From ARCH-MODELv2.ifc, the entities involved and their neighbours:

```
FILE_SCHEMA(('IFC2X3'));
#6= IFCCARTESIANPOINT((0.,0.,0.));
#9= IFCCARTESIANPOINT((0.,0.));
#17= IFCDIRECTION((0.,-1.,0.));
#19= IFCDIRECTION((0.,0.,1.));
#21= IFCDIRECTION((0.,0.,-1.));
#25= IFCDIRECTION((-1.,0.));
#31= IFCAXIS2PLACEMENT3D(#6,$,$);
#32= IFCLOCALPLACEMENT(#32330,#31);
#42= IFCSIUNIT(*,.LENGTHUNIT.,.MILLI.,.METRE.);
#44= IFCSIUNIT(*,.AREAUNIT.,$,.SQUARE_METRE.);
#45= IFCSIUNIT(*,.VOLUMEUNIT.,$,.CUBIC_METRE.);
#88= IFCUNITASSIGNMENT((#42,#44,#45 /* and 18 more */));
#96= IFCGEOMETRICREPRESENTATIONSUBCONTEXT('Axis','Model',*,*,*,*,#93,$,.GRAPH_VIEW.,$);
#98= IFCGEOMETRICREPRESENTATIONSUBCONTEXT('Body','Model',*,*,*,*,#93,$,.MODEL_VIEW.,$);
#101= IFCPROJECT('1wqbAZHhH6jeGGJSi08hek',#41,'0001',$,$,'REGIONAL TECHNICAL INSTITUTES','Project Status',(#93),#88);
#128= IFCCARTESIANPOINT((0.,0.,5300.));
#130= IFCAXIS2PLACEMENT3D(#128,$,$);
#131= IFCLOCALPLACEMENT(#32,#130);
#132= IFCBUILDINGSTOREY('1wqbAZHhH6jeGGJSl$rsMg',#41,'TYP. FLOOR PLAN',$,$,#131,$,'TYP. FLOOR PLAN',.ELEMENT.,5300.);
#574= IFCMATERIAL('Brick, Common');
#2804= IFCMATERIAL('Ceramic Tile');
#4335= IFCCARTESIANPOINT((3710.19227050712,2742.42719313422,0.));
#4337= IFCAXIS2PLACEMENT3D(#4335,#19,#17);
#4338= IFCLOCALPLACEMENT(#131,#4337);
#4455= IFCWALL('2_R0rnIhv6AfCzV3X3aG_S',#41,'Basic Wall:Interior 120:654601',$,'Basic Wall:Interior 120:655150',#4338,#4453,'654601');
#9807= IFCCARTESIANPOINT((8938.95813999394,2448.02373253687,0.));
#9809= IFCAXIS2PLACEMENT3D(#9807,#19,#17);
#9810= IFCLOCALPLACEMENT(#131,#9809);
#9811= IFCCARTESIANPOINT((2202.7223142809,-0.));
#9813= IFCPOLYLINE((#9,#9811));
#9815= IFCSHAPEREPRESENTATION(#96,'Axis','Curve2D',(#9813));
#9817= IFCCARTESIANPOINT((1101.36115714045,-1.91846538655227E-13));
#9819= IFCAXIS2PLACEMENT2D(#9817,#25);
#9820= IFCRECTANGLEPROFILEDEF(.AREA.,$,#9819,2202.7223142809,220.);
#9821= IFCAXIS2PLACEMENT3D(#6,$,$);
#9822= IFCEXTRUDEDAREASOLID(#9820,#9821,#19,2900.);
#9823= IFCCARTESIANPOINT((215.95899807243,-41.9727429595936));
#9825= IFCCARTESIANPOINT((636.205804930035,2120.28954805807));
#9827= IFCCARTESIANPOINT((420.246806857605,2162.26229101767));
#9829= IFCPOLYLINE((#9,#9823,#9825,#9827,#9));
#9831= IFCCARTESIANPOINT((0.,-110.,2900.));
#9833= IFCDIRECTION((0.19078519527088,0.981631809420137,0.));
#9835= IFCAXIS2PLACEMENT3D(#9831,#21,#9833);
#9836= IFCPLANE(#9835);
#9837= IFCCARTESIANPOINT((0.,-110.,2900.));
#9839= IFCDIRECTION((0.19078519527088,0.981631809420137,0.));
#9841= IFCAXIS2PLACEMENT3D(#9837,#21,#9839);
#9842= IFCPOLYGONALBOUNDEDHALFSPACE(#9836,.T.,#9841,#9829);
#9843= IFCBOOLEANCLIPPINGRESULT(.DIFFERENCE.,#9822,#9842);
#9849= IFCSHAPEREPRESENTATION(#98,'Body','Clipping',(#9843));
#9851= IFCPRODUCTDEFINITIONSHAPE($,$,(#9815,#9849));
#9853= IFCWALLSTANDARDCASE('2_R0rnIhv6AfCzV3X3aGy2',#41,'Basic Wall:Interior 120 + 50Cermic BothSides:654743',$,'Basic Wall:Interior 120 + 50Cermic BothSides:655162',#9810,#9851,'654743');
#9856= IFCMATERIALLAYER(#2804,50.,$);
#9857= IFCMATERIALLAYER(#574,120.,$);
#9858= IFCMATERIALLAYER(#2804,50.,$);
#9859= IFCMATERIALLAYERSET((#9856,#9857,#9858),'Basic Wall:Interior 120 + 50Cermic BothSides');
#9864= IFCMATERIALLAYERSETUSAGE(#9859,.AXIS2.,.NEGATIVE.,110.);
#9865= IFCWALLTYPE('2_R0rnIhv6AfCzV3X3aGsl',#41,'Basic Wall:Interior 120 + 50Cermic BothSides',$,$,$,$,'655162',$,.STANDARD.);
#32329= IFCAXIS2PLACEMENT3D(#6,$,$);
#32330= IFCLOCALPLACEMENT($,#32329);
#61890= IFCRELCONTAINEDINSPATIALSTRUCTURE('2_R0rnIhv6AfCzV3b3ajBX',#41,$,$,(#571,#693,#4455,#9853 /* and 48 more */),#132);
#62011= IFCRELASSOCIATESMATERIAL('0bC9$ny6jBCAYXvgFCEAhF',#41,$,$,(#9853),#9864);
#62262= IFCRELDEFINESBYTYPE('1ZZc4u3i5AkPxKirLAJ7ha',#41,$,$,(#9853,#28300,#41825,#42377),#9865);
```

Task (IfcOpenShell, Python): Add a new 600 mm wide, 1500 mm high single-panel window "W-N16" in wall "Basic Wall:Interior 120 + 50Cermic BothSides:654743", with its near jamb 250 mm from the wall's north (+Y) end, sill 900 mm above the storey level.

```python
import numpy as np
import ifcopenshell
import ifcopenshell.api.feature
import ifcopenshell.api.geometry
import ifcopenshell.api.root
import ifcopenshell.api.spatial
import ifcopenshell.api.type
import ifcopenshell.geom
import ifcopenshell.util.element
import ifcopenshell.util.placement
import ifcopenshell.util.representation
import ifcopenshell.util.shape
import ifcopenshell.util.unit

model = ifcopenshell.open("ARCH-MODELv2.ifc")
unit_scale = ifcopenshell.util.unit.calculate_unit_scale(model)
settings = ifcopenshell.geom.settings()


def volume(element):
    """Net volume in cubic metres, openings subtracted."""
    shape = ifcopenshell.geom.create_shape(settings, element)
    return ifcopenshell.util.shape.get_volume(shape.geometry)


wall = model.by_guid("2_R0rnIhv6AfCzV3X3aGy2")
storey = ifcopenshell.util.element.get_container(wall, ifc_class="IfcBuildingStorey")
context = ifcopenshell.util.representation.get_context(model, "Model", "Body", "MODEL_VIEW")
before = volume(wall)

width, height, from_end, sill = 0.6, 1.5, 0.25, 0.9  # metres

# The wall runs along its own X axis, and the end named is its -X end.
wall_shape = ifcopenshell.geom.create_shape(settings, wall)
x, y, z = ifcopenshell.util.shape.get_vertices(wall_shape.geometry).T
start = x.min() + from_end
face, thickness = float(y.min()), float(y.max() - y.min())
wall_matrix = ifcopenshell.util.placement.get_local_placement(wall.ObjectPlacement)
level = ifcopenshell.util.placement.get_local_placement(storey.ObjectPlacement)[2, 3]


def in_wall(x, y):
    """Placement at x, y metres in the wall's axes, at sill height."""
    matrix = wall_matrix.copy()
    matrix[:, 3] = wall_matrix @ np.array([x / unit_scale, y / unit_scale, 0.0, 1.0])
    matrix[2, 3] = level + sill / unit_scale
    return matrix


# Opening: a box that overshoots both wall faces by 50 mm.
opening = ifcopenshell.api.root.create_entity(model, ifc_class="IfcOpeningElement")
box = ifcopenshell.api.geometry.add_wall_representation(
    model, context=context, length=width, height=height, thickness=thickness + 0.1
)
ifcopenshell.api.geometry.assign_representation(model, product=opening, representation=box)
ifcopenshell.api.geometry.edit_object_placement(model, product=opening, matrix=in_wall(start, face - 0.05), is_si=False)
ifcopenshell.api.feature.add_feature(model, feature=opening, element=wall)

window = ifcopenshell.api.root.create_entity(model, ifc_class="IfcWindow", name="W-N16")
window.OverallWidth, window.OverallHeight = width / unit_scale, height / unit_scale
body = ifcopenshell.api.geometry.add_window_representation(
    model,
    context=context,
    overall_width=window.OverallWidth,
    overall_height=window.OverallHeight,
    partition_type="SINGLE_PANEL",
)
ifcopenshell.api.geometry.assign_representation(model, product=window, representation=body)
ifcopenshell.api.spatial.assign_container(model, products=[window], relating_structure=storey)
fills = ifcopenshell.api.feature.add_filling(model, opening=opening, element=window)
fills.OwnerHistory = window.OwnerHistory  # required in IFC2X3

# IFC2X3 keeps the operation on the window style.
style = ifcopenshell.api.root.create_entity(model, ifc_class="IfcWindowStyle", name="W-N16")
style.OperationType, style.ConstructionType = "SINGLE_PANEL", "NOTDEFINED"
style.ParameterTakesPrecedence = style.Sizeable = False
ifcopenshell.api.type.assign_type(model, related_objects=[window], relating_type=style)

# Centre the window in the wall's thickness.
ifcopenshell.api.geometry.edit_object_placement(model, product=window, matrix=in_wall(start, face), is_si=False)
window_shape = ifcopenshell.geom.create_shape(settings, window)
depth = ifcopenshell.util.shape.get_vertices(window_shape.geometry)[:, 1]
offset = face + thickness / 2 - (depth.min() + depth.max()) / 2
ifcopenshell.api.geometry.edit_object_placement(model, product=window, matrix=in_wall(start, offset), is_si=False)

after = volume(wall)

print(f"wall volume {before:.3f} -> {after:.3f} m3")

model.write("ARCH-MODELv2-out.ifc")
```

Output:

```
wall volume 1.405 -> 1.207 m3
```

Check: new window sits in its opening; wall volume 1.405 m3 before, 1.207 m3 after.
